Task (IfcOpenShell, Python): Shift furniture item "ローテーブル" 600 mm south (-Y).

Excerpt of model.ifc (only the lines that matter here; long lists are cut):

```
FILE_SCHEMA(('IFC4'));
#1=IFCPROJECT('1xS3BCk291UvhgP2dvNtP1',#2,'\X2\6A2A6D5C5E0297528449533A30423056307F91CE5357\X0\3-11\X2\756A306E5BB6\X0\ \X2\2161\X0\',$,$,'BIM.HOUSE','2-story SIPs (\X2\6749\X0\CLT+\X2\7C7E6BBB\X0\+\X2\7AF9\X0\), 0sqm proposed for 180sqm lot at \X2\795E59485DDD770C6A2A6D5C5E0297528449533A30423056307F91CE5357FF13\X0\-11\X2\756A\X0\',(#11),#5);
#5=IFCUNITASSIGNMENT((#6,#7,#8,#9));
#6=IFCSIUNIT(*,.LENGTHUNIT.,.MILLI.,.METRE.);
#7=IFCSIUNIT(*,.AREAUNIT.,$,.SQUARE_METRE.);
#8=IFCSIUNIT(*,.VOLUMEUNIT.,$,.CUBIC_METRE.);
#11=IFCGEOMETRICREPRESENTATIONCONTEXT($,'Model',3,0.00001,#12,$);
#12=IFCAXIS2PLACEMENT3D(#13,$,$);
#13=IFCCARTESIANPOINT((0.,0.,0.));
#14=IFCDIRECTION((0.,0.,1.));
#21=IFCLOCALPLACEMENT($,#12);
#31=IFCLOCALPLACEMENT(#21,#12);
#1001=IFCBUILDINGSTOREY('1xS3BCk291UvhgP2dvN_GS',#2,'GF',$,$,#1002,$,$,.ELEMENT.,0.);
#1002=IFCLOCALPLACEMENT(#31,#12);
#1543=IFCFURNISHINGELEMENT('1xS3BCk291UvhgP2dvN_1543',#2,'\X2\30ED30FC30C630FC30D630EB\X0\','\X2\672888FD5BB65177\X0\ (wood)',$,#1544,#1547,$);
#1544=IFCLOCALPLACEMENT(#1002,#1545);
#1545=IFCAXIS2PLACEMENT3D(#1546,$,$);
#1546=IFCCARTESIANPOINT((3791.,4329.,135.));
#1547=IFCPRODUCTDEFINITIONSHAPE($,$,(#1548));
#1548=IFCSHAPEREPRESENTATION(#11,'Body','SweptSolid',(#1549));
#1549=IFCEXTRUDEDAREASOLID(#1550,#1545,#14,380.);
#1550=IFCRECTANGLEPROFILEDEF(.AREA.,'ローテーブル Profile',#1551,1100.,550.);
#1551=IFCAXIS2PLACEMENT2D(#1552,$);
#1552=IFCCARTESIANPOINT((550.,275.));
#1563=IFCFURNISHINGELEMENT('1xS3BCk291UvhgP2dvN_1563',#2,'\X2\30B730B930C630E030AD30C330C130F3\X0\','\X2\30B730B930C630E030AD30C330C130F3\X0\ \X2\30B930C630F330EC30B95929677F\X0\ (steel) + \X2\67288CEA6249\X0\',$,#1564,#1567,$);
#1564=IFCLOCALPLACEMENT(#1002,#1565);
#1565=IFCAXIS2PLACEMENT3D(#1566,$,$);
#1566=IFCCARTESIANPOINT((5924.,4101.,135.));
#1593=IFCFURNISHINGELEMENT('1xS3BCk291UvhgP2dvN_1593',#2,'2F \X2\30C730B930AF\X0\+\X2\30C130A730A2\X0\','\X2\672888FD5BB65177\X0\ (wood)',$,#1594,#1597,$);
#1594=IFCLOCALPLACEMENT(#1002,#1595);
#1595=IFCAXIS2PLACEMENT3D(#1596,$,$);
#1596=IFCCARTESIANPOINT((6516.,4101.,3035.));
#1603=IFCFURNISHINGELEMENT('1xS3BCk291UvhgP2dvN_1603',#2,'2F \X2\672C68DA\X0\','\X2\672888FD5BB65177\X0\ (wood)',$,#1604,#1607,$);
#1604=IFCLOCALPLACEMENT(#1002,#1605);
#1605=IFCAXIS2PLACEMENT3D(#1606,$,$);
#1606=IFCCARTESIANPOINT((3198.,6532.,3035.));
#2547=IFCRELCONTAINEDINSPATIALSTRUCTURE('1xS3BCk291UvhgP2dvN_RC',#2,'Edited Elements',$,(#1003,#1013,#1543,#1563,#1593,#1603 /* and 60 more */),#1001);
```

```python
import ifcopenshell
import ifcopenshell.api.geometry
import ifcopenshell.util.placement

model = ifcopenshell.open("model.ifc")

item = model.by_guid("1xS3BCk291UvhgP2dvN_1543")
matrix = ifcopenshell.util.placement.get_local_placement(item.ObjectPlacement)
matrix[1, 3] -= 600.0
ifcopenshell.api.geometry.edit_object_placement(model, product=item, matrix=matrix, is_si=False)

print(ifcopenshell.util.placement.get_local_placement(item.ObjectPlacement).round(3) + 0.0)

model.write("model-out.ifc")
```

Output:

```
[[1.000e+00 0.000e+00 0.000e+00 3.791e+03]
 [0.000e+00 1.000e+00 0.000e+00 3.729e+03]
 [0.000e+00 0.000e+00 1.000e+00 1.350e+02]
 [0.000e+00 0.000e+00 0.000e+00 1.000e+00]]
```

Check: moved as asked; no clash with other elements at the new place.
